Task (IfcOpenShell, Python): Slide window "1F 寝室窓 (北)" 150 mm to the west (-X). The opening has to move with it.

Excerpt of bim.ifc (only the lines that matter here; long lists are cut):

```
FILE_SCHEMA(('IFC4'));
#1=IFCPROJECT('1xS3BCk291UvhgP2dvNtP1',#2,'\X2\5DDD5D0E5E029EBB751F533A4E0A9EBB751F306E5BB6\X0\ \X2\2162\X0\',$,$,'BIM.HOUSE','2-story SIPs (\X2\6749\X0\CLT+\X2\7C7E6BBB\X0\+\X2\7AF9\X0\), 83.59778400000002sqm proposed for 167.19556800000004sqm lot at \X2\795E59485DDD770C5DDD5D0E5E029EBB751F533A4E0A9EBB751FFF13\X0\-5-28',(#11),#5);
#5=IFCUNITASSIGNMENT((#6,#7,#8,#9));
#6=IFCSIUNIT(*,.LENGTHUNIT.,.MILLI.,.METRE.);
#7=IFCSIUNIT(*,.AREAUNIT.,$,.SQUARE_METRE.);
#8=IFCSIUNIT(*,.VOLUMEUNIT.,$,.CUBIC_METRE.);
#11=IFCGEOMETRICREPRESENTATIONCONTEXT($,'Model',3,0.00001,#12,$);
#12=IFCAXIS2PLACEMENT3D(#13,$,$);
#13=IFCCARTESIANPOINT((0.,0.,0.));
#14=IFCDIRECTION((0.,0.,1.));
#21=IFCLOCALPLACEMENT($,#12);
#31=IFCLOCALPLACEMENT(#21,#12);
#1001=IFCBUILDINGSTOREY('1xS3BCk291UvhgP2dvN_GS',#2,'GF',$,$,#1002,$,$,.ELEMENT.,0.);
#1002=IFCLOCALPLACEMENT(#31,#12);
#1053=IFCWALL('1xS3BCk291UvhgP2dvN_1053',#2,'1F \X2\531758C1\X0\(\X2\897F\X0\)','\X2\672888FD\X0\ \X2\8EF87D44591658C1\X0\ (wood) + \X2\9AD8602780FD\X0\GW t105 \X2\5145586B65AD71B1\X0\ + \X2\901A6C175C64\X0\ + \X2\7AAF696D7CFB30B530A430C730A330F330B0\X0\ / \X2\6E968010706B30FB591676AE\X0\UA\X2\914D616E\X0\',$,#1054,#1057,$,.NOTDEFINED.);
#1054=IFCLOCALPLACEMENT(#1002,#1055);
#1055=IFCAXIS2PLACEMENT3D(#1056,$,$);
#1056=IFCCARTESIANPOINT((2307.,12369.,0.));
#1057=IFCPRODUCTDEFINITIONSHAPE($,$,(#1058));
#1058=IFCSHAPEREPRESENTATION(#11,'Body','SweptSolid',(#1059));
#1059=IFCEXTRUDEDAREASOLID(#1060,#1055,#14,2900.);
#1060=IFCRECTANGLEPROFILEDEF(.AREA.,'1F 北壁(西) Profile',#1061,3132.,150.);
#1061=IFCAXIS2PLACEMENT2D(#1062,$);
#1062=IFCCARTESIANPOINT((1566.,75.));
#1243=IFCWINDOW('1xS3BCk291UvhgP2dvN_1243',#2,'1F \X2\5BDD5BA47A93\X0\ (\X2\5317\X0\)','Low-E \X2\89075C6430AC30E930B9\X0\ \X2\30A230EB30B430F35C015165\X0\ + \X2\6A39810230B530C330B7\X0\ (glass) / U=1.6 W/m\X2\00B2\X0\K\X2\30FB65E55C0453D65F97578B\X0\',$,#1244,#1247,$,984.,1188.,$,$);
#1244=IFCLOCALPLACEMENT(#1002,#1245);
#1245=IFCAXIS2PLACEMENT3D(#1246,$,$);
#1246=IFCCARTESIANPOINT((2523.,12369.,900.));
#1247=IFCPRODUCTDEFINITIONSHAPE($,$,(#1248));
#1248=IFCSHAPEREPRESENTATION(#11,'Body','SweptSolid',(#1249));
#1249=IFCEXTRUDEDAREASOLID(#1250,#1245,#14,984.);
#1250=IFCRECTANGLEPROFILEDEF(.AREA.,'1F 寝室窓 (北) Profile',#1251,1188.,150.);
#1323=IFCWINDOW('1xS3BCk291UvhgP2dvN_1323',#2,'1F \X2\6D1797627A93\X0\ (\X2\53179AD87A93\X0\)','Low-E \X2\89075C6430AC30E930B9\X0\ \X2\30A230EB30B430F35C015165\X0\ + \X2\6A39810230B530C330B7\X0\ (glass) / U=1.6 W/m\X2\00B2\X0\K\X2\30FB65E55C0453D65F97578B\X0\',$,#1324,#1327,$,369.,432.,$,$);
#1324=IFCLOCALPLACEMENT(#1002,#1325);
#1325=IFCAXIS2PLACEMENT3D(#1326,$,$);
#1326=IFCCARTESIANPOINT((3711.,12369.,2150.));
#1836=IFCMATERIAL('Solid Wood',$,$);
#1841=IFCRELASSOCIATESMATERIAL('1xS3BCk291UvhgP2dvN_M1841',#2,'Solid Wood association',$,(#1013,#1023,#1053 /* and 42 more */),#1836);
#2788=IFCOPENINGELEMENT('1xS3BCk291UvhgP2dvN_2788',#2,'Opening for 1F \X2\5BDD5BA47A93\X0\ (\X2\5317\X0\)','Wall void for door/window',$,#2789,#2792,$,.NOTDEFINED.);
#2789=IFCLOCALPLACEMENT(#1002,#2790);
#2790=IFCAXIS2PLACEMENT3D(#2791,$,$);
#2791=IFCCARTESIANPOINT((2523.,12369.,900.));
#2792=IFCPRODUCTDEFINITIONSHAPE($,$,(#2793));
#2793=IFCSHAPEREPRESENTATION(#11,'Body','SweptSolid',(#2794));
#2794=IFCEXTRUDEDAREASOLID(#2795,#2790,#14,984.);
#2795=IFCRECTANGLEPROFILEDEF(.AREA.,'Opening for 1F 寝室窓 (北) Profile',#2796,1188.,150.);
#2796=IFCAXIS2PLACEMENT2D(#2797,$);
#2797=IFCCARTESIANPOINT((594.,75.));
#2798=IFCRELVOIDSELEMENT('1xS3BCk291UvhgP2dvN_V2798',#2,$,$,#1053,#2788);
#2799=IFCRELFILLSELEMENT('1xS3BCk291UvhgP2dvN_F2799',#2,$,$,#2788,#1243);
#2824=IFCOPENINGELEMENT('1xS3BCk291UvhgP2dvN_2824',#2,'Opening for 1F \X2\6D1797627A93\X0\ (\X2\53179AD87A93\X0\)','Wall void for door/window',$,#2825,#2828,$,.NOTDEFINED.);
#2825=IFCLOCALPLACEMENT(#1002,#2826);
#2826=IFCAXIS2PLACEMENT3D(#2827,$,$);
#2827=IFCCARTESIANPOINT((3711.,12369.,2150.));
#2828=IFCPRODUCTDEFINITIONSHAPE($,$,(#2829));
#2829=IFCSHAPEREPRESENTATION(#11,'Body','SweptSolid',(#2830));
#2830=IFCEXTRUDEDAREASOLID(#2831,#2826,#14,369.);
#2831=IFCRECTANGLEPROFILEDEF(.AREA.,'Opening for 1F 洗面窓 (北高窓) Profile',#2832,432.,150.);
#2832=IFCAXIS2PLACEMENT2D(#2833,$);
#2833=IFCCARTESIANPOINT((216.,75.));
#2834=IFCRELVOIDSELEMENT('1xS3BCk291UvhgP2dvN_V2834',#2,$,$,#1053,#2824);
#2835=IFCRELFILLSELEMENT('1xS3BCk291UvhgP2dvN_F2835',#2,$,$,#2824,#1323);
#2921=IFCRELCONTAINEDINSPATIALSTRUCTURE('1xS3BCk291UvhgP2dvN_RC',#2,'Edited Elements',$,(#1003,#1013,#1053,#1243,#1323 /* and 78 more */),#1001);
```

```python
import ifcopenshell
import ifcopenshell.api.geometry
import ifcopenshell.util.placement
import ifcopenshell.util.unit

model = ifcopenshell.open("bim.ifc")
unit_scale = ifcopenshell.util.unit.calculate_unit_scale(model)

window = model.by_guid("1xS3BCk291UvhgP2dvN_1243")
opening = window.FillsVoids[0].RelatingOpeningElement
wall = opening.VoidsElements[0].RelatingBuildingElement

wall_matrix = ifcopenshell.util.placement.get_local_placement(wall.ObjectPlacement)
shift = wall_matrix[:3, 0] * -0.15 / unit_scale
before = ifcopenshell.util.placement.get_local_placement(window.ObjectPlacement)[:3, 3].copy()

# The window is not placed relative to its opening, so move both.
for product in (opening, window):
    matrix = ifcopenshell.util.placement.get_local_placement(product.ObjectPlacement)
    matrix[:3, 3] += shift
    ifcopenshell.api.geometry.edit_object_placement(model, product=product, matrix=matrix, is_si=False)

after = ifcopenshell.util.placement.get_local_placement(window.ObjectPlacement)[:3, 3]
print("window moved by", (after - before).round(3) + 0.0)

model.write("bim_v2.ifc")
```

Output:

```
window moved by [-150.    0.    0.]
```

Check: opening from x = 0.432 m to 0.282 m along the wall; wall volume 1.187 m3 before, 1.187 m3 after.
